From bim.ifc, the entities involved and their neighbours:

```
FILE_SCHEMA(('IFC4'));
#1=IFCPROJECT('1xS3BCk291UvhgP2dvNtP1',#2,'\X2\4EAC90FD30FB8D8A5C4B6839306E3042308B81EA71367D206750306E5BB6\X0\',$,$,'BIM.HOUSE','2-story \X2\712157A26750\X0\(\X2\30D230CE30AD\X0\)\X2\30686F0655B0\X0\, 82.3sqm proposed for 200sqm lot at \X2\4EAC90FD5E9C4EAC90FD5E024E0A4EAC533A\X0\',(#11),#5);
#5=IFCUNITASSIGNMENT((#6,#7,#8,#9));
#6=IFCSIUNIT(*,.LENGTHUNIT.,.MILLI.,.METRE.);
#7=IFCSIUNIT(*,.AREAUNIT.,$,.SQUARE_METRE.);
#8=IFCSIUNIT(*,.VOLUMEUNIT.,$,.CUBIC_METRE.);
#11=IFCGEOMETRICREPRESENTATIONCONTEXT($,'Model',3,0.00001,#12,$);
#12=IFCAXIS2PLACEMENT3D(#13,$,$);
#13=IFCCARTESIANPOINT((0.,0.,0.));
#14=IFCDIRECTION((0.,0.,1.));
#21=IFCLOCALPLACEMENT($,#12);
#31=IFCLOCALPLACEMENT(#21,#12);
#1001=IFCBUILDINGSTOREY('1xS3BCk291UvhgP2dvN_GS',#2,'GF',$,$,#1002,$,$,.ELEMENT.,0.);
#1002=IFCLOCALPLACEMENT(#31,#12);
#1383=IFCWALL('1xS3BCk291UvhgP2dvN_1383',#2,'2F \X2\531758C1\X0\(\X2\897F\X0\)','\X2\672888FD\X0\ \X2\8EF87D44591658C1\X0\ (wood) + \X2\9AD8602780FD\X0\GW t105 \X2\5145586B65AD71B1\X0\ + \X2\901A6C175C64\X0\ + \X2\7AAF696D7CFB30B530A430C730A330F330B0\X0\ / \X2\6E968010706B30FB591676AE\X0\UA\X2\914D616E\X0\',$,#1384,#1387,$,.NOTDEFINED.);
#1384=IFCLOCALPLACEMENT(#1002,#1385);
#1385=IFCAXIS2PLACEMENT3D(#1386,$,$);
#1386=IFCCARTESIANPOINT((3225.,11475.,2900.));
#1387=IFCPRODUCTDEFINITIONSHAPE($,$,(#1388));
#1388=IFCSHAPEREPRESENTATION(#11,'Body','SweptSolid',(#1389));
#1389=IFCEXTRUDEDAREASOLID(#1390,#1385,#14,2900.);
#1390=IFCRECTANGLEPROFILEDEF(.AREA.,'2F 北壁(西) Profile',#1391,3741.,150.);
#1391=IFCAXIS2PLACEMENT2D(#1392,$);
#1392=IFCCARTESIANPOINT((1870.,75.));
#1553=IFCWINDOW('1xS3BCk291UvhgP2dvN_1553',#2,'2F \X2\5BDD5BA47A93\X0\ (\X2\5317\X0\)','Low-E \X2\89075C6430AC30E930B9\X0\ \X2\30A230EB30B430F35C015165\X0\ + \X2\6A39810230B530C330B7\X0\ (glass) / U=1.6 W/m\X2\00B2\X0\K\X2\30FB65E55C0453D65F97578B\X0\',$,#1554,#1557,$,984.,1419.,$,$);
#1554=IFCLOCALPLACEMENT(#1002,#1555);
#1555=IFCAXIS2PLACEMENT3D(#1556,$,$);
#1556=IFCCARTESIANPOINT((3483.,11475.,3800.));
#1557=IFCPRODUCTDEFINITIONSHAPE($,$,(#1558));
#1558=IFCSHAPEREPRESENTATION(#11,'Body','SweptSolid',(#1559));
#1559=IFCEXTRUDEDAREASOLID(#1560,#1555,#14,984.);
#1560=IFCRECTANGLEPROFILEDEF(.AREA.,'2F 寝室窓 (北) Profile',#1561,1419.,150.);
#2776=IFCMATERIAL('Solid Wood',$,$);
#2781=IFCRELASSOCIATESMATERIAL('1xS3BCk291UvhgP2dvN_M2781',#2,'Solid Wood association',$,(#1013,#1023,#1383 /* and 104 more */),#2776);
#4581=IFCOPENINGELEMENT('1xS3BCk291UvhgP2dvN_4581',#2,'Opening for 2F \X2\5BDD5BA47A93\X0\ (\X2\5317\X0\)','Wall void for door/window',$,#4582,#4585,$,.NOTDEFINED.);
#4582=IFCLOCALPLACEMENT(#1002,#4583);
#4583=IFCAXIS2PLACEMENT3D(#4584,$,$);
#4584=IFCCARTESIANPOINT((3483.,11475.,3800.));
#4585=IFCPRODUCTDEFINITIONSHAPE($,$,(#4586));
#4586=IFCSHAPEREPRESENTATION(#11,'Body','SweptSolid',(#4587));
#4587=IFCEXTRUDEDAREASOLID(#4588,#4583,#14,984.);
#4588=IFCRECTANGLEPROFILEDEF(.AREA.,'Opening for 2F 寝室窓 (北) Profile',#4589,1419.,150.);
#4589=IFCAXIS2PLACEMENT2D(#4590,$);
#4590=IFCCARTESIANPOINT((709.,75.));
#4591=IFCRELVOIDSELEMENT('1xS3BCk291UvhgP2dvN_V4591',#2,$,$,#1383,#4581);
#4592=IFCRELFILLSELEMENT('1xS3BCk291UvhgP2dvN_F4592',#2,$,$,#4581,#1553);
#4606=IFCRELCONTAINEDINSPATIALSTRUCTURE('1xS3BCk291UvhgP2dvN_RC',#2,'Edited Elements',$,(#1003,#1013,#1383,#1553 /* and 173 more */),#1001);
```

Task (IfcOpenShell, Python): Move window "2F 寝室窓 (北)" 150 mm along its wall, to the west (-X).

```python
import ifcopenshell
import ifcopenshell.api.geometry
import ifcopenshell.util.placement

model = ifcopenshell.open("bim.ifc")

window = model.by_guid("1xS3BCk291UvhgP2dvN_1553")
opening = window.FillsVoids[0].RelatingOpeningElement
wall = opening.VoidsElements[0].RelatingBuildingElement

wall_matrix = ifcopenshell.util.placement.get_local_placement(wall.ObjectPlacement)
shift = wall_matrix[:3, 0] * -150.0
before = ifcopenshell.util.placement.get_local_placement(window.ObjectPlacement)[:3, 3].copy()

# The window is not placed relative to its opening, so move both.
for product in (opening, window):
    matrix = ifcopenshell.util.placement.get_local_placement(product.ObjectPlacement)
    matrix[:3, 3] += shift
    ifcopenshell.api.geometry.edit_object_placement(model, product=product, matrix=matrix, is_si=False)

after = ifcopenshell.util.placement.get_local_placement(window.ObjectPlacement)[:3, 3]
print("window moved by", (after - before).round(3) + 0.0)

model.write("bim_rev.ifc")
```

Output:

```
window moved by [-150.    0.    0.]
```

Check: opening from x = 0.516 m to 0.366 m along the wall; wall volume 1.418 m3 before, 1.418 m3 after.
